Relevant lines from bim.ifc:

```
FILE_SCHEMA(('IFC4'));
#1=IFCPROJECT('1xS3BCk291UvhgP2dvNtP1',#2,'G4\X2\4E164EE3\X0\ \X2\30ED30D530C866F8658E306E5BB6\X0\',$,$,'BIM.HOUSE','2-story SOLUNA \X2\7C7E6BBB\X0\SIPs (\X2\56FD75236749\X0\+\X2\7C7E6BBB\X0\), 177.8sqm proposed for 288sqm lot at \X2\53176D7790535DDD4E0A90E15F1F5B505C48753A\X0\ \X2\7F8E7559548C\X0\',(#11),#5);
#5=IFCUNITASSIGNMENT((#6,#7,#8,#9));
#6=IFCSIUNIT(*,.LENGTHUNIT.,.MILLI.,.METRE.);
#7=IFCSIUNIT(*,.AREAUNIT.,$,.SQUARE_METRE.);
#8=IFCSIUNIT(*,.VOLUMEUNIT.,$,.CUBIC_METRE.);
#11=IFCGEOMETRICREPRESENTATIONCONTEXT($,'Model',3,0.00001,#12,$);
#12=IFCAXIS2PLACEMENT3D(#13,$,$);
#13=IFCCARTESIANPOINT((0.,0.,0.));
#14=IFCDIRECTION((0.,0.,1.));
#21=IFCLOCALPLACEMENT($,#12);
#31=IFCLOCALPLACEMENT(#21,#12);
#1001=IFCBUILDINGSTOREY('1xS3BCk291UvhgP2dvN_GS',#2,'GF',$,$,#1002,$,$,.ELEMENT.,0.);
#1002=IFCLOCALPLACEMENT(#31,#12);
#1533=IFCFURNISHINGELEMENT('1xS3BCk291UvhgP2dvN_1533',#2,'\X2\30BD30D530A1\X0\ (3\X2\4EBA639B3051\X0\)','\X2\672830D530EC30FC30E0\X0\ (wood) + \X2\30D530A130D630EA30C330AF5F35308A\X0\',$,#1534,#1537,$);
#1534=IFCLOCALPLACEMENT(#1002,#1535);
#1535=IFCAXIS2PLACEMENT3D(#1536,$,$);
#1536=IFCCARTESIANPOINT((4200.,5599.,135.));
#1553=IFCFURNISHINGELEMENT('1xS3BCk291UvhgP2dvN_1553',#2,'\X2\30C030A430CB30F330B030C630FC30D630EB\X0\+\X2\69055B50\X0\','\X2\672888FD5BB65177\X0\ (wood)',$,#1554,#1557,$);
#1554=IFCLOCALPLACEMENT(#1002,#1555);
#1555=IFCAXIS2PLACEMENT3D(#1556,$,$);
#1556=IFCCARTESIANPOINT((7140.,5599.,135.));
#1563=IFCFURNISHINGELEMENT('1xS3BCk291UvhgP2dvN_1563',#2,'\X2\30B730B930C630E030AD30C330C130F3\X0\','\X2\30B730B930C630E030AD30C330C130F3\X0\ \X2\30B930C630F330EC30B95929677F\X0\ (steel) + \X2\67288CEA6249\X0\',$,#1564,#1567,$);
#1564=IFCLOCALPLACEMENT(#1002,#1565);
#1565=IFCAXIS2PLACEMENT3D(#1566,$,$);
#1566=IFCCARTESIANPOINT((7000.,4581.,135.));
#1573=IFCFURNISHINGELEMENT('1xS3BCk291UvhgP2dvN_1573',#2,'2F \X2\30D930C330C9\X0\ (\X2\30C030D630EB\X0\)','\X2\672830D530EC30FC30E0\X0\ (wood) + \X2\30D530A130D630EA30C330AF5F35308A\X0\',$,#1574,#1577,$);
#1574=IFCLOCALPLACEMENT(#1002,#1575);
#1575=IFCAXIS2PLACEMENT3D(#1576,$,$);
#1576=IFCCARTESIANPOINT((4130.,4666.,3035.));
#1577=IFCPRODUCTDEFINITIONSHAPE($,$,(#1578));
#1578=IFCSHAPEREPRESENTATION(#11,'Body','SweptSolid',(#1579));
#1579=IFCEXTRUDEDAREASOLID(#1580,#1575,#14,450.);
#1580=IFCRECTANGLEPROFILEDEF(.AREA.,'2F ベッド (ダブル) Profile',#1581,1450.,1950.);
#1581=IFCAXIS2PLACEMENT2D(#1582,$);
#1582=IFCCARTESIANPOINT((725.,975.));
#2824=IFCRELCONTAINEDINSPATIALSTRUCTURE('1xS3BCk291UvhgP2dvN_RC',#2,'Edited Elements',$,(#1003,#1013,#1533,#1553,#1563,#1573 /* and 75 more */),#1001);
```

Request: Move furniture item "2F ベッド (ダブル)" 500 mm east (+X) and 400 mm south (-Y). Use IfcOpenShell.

```python
import ifcopenshell
import ifcopenshell.api.geometry
import ifcopenshell.util.placement
import ifcopenshell.util.unit

model = ifcopenshell.open("bim.ifc")
unit_scale = ifcopenshell.util.unit.calculate_unit_scale(model)

item = model.by_guid("1xS3BCk291UvhgP2dvN_1573")
matrix = ifcopenshell.util.placement.get_local_placement(item.ObjectPlacement)
matrix[0, 3] += 0.5 / unit_scale
matrix[1, 3] -= 0.4 / unit_scale
ifcopenshell.api.geometry.edit_object_placement(model, product=item, matrix=matrix, is_si=False)

print(ifcopenshell.util.placement.get_local_placement(item.ObjectPlacement).round(3) + 0.0)

model.write("bim_updated.ifc")
```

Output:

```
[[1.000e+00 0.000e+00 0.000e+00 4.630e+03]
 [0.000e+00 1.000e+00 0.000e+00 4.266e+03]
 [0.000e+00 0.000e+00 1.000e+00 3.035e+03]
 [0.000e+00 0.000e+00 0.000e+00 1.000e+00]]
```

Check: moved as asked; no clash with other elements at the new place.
